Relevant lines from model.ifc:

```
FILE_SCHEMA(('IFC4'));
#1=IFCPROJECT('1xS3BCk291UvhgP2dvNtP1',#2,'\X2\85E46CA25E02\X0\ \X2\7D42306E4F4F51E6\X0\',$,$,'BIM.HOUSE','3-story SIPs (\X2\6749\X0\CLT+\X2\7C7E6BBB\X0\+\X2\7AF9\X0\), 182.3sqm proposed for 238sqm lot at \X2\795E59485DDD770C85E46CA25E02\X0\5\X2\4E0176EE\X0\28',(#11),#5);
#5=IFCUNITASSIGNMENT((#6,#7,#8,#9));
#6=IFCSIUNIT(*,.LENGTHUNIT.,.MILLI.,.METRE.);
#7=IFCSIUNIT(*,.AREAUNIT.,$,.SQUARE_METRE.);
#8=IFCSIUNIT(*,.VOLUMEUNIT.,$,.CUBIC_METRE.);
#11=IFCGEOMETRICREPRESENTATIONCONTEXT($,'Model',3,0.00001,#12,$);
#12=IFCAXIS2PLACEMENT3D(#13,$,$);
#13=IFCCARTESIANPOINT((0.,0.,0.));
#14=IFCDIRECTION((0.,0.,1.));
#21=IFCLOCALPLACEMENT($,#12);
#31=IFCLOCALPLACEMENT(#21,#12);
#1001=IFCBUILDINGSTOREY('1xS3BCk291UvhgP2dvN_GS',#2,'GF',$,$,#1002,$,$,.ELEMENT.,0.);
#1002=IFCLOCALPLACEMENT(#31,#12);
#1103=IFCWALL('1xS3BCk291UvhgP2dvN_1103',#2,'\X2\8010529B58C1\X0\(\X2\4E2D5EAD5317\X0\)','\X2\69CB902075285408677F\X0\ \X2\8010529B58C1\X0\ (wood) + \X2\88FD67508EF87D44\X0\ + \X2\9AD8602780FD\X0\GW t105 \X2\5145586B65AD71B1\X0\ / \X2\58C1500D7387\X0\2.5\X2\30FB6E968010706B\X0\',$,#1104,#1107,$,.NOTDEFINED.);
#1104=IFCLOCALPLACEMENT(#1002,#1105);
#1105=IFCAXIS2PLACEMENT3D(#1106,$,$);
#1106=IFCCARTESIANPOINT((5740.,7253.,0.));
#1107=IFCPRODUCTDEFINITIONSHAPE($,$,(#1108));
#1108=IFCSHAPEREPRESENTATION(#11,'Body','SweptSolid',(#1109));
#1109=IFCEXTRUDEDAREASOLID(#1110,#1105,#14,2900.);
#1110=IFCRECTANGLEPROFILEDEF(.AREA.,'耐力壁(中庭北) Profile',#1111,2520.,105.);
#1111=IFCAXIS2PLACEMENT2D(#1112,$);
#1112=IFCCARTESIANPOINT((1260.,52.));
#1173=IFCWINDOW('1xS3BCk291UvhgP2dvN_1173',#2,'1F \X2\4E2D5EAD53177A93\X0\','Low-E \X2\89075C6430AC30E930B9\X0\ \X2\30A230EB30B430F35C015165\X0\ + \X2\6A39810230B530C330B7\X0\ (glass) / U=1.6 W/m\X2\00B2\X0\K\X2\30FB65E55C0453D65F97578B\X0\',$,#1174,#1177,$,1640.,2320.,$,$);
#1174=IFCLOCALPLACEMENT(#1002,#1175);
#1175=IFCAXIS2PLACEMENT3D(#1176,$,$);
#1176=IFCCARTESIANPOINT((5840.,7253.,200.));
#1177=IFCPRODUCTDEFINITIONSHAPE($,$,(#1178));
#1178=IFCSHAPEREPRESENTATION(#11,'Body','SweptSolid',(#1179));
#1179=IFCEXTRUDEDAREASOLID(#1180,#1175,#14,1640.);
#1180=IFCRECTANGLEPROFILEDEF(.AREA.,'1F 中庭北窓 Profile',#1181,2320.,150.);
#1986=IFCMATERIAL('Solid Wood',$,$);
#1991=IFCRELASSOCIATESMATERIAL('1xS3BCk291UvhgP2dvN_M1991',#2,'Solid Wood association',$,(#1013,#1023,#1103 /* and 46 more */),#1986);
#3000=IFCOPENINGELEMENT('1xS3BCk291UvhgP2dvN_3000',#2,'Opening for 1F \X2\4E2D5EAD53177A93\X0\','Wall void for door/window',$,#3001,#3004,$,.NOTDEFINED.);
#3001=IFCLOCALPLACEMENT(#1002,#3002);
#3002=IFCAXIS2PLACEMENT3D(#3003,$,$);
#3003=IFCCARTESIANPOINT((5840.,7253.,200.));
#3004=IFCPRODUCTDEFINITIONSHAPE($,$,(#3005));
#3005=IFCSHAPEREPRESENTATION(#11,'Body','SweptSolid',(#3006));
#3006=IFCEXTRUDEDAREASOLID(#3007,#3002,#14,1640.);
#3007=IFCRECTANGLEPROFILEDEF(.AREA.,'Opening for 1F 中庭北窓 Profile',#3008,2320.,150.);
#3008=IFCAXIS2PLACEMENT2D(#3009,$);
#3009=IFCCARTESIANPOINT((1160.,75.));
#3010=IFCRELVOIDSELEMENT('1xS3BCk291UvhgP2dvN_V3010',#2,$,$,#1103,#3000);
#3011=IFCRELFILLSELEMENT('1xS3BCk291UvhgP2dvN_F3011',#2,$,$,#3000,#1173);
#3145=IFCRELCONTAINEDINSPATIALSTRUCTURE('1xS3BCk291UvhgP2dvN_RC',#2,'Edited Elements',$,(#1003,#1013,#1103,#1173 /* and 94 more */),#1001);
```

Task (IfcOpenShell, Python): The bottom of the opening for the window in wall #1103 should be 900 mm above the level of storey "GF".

```python
import numpy as np
import ifcopenshell
import ifcopenshell.api.geometry
import ifcopenshell.geom
import ifcopenshell.util.element
import ifcopenshell.util.placement
import ifcopenshell.util.shape
import ifcopenshell.util.unit

model = ifcopenshell.open("model.ifc")
unit_scale = ifcopenshell.util.unit.calculate_unit_scale(model)

window = model.by_id(1173)
opening = window.FillsVoids[0].RelatingOpeningElement
storey = ifcopenshell.util.element.get_container(window, ifc_class="IfcBuildingStorey")
level = ifcopenshell.util.placement.get_local_placement(storey.ObjectPlacement)[2, 3]

# The opening's origin need not be at the sill, so measure its lowest point.
shape = ifcopenshell.geom.create_shape(ifcopenshell.geom.settings(), opening)
bottom = ifcopenshell.util.shape.get_shape_bottom_elevation(shape, shape.geometry) / unit_scale
dz = level + 0.9 / unit_scale - bottom

shift = np.array([0.0, 0.0, dz])
# The window is not placed relative to its opening, so move both.
for product in (opening, window):
    matrix = ifcopenshell.util.placement.get_local_placement(product.ObjectPlacement)
    matrix[:3, 3] += shift
    ifcopenshell.api.geometry.edit_object_placement(model, product=product, matrix=matrix, is_si=False)

print(f"moved by {dz * unit_scale:+.3f} m")

model.write("model-out.ifc")
```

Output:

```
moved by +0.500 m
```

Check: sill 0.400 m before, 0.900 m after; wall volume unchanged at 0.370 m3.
